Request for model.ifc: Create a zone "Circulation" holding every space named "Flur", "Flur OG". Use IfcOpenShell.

First a look at what the model holds.

```python
import ifcopenshell

model = ifcopenshell.open("model.ifc")
print(model.schema)
seen = {}
for space in model.by_type("IfcSpace"):
    seen[space.LongName] = seen.get(space.LongName, 0) + 1
for name, count in sorted(seen.items(), key=str):
    print(count, "x", name)
print("zones:", [z.Name for z in model.by_type("IfcZone")][:20])
```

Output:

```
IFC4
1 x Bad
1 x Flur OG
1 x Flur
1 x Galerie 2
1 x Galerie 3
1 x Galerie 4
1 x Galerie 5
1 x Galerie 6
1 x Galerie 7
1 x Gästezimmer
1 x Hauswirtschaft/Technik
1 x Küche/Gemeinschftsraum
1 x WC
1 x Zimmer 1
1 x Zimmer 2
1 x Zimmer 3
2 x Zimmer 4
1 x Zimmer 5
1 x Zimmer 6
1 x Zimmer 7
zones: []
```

```python
import ifcopenshell
import ifcopenshell.api.group
import ifcopenshell.api.root

model = ifcopenshell.open("model.ifc")

names = {"Flur", "Flur OG"}
spaces = [s for s in model.by_type("IfcSpace") if s.LongName in names]

zone = ifcopenshell.api.root.create_entity(model, ifc_class="IfcZone", name="Circulation")
ifcopenshell.api.group.assign_group(model, products=spaces, group=zone)
print(len(spaces), "spaces in", zone.Name)

model.write("model_v2.ifc")
```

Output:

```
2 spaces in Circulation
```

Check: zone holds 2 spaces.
